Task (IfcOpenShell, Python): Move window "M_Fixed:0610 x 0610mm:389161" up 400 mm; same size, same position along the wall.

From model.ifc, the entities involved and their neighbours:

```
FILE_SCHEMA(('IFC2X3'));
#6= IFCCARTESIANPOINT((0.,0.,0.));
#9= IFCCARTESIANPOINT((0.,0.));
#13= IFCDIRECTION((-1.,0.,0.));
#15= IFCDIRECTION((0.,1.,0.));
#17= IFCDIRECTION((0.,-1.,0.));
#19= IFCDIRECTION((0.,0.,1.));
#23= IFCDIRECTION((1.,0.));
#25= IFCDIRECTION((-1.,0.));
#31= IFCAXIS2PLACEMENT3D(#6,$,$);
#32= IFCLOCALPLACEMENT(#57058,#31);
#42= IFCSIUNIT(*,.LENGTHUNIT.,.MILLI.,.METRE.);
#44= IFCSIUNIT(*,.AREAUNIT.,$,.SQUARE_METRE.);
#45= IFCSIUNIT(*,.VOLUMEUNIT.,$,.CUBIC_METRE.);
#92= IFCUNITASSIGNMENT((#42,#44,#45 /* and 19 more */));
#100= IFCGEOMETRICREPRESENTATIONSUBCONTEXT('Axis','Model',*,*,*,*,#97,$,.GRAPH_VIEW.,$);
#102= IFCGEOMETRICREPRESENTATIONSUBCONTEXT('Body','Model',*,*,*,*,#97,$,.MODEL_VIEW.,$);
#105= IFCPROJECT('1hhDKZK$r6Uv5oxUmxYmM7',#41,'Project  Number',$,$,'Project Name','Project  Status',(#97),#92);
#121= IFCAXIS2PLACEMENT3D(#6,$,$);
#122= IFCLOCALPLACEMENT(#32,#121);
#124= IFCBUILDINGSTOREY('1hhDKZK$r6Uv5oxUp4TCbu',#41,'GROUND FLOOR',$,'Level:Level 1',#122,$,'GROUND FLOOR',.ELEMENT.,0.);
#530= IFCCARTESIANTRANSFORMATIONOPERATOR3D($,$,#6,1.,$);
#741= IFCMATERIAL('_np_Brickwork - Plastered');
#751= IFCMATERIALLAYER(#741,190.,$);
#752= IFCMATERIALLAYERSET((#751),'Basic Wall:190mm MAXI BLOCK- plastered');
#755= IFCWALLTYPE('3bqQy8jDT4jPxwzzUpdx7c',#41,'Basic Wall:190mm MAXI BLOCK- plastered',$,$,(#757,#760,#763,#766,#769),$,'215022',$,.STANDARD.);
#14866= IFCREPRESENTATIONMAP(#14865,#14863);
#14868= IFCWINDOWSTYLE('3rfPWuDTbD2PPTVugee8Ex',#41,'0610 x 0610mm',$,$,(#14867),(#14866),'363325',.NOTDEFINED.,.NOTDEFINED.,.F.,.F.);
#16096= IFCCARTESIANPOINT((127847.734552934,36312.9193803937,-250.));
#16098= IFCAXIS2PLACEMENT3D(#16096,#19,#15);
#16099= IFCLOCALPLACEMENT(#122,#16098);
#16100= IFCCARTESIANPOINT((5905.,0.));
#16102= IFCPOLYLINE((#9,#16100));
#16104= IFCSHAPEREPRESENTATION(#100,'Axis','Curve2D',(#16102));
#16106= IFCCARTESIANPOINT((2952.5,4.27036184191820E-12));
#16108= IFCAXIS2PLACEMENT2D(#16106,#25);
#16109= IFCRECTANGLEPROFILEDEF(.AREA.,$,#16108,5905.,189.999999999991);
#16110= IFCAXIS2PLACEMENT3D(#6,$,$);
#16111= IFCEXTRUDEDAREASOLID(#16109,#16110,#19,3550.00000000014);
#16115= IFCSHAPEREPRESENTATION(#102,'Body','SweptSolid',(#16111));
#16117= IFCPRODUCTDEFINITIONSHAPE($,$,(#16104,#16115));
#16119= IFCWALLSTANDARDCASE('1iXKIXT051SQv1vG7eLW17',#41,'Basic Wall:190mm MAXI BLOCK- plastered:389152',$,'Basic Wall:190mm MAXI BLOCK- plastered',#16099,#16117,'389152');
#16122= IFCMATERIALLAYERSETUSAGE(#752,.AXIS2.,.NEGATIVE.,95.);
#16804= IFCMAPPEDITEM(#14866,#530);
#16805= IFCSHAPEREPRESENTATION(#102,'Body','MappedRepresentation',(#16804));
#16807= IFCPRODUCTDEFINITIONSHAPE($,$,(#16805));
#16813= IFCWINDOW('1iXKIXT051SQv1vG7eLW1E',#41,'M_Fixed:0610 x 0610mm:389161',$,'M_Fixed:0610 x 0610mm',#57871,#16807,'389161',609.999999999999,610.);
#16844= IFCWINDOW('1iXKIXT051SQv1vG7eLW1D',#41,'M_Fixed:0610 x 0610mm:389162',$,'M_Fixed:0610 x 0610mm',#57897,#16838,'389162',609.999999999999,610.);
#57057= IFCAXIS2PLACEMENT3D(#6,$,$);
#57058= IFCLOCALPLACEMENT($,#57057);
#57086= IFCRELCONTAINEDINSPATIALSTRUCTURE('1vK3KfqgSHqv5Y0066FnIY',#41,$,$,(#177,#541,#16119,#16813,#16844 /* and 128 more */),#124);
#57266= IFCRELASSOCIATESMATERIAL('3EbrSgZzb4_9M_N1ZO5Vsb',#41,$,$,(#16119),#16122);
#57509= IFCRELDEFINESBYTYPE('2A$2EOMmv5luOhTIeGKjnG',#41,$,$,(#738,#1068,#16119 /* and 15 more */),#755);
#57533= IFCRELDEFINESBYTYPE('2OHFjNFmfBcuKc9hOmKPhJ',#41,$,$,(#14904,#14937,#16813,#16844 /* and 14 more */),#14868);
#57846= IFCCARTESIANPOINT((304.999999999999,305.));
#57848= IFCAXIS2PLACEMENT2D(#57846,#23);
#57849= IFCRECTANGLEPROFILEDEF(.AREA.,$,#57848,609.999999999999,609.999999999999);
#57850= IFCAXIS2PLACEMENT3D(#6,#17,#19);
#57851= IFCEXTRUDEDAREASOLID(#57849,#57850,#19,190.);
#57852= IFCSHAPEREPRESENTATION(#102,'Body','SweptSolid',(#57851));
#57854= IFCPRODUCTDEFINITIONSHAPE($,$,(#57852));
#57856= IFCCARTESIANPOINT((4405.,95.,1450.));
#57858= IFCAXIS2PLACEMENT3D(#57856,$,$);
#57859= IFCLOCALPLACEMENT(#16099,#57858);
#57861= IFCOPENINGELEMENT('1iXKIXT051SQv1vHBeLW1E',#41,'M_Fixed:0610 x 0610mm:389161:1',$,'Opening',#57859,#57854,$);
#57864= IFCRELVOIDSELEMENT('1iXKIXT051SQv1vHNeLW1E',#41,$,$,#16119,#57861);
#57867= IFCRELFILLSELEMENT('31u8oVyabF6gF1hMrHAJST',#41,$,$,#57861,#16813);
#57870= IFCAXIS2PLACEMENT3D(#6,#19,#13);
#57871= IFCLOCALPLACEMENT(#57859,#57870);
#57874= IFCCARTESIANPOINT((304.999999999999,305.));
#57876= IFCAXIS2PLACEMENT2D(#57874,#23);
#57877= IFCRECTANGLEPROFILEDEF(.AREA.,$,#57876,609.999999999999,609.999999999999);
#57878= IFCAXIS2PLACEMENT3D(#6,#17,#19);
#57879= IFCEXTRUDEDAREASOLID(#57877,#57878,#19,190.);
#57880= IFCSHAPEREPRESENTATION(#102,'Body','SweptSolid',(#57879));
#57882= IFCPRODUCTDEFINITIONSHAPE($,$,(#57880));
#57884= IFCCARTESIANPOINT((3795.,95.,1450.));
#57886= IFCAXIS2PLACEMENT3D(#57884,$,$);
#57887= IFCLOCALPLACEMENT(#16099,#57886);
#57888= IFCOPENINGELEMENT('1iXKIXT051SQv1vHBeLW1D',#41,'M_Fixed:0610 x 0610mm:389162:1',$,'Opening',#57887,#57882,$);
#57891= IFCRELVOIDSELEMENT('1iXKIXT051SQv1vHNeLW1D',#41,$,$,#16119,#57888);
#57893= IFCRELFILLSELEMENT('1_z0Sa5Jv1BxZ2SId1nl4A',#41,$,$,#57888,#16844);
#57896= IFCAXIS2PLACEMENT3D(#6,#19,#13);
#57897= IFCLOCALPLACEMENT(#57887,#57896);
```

```python
import numpy as np
import ifcopenshell
import ifcopenshell.api.geometry
import ifcopenshell.util.placement
import ifcopenshell.util.unit

model = ifcopenshell.open("model.ifc")
unit_scale = ifcopenshell.util.unit.calculate_unit_scale(model)

window = model.by_guid("1iXKIXT051SQv1vG7eLW1E")
opening = window.FillsVoids[0].RelatingOpeningElement
dz = 400.0

shift = np.array([0.0, 0.0, dz])
# The window is placed relative to its opening, so it follows when the opening moves.
matrix = ifcopenshell.util.placement.get_local_placement(opening.ObjectPlacement)
matrix[:3, 3] += shift
ifcopenshell.api.geometry.edit_object_placement(
    model, product=opening, matrix=matrix, is_si=False, should_transform_children=True
)

print(f"moved by {dz * unit_scale:+.3f} m")

model.write("model_rev.ifc")
```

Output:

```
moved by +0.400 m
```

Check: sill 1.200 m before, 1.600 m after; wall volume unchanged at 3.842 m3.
